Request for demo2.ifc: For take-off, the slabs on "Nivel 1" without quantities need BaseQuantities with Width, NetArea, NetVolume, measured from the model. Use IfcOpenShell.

First a look at what the model holds.

```python
import ifcopenshell
import ifcopenshell.util.element
import ifcopenshell.util.unit

model = ifcopenshell.open("demo2.ifc")
print(model.schema)
for unit_type in ("LENGTHUNIT", "AREAUNIT", "VOLUMEUNIT"):
    print(unit_type, ifcopenshell.util.unit.calculate_unit_scale(model, unit_type))
storey = next(s for s in model.by_type("IfcBuildingStorey") if s.Name == "Nivel 1")
slabs = [e for e in ifcopenshell.util.element.get_decomposition(storey) if e.is_a("IfcSlab")]
for e in sorted(slabs, key=lambda e: e.id()):
    print(e.id(), e.is_a(), e.Name, list(ifcopenshell.util.element.get_psets(e, qtos_only=True)), sep=" | ")
```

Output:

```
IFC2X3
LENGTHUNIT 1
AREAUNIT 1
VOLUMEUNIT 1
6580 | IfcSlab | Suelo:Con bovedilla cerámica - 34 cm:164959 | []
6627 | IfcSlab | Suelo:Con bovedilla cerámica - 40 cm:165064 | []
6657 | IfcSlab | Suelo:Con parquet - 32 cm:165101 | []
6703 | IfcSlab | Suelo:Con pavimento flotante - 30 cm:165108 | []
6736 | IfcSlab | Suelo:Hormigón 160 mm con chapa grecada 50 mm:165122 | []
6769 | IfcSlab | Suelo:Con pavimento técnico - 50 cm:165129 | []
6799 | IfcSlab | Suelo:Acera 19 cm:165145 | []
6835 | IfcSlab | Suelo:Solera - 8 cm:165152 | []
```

```python
import ifcopenshell
import ifcopenshell.api.pset
import ifcopenshell.geom
import ifcopenshell.util.element
import ifcopenshell.util.shape
import ifcopenshell.util.unit

model = ifcopenshell.open("demo2.ifc")
unit_scale = ifcopenshell.util.unit.calculate_unit_scale(model)
area_scale = ifcopenshell.util.unit.calculate_unit_scale(model, "AREAUNIT")
volume_scale = ifcopenshell.util.unit.calculate_unit_scale(model, "VOLUMEUNIT")
settings = ifcopenshell.geom.settings()

storey = next(s for s in model.by_type("IfcBuildingStorey") if s.Name == "Nivel 1")
slabs = [e for e in ifcopenshell.util.element.get_decomposition(storey) if e.is_a("IfcSlab")]

for e in sorted(slabs, key=lambda e: e.id()):
    if ifcopenshell.util.element.get_psets(e, qtos_only=True, should_inherit=False):
        continue
    # Geometry comes back in metres, in the element's own axes.
    shape = ifcopenshell.geom.create_shape(settings, e)
    values = {
        "Width": ifcopenshell.util.shape.get_z(shape.geometry) / unit_scale,
        "NetArea": ifcopenshell.util.shape.get_footprint_area(shape.geometry) / area_scale,
        "NetVolume": ifcopenshell.util.shape.get_volume(shape.geometry) / volume_scale,
    }
    qto = ifcopenshell.api.pset.add_qto(model, product=e, name="BaseQuantities")
    ifcopenshell.api.pset.edit_qto(model, qto=qto, properties=values)
    print(e.id(), {k: round(v, 3) for k, v in values.items()})

model.write("demo2_edited.ifc")
```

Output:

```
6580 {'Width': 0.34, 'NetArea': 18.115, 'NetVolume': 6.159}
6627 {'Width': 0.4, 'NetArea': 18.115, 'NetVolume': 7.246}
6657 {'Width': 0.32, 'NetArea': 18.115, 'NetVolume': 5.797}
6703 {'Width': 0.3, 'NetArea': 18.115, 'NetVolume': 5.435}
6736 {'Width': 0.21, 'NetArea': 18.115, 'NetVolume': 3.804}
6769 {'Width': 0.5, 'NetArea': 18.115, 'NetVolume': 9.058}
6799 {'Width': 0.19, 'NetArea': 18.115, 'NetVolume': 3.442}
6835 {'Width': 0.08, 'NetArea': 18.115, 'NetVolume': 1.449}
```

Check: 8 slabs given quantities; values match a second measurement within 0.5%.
